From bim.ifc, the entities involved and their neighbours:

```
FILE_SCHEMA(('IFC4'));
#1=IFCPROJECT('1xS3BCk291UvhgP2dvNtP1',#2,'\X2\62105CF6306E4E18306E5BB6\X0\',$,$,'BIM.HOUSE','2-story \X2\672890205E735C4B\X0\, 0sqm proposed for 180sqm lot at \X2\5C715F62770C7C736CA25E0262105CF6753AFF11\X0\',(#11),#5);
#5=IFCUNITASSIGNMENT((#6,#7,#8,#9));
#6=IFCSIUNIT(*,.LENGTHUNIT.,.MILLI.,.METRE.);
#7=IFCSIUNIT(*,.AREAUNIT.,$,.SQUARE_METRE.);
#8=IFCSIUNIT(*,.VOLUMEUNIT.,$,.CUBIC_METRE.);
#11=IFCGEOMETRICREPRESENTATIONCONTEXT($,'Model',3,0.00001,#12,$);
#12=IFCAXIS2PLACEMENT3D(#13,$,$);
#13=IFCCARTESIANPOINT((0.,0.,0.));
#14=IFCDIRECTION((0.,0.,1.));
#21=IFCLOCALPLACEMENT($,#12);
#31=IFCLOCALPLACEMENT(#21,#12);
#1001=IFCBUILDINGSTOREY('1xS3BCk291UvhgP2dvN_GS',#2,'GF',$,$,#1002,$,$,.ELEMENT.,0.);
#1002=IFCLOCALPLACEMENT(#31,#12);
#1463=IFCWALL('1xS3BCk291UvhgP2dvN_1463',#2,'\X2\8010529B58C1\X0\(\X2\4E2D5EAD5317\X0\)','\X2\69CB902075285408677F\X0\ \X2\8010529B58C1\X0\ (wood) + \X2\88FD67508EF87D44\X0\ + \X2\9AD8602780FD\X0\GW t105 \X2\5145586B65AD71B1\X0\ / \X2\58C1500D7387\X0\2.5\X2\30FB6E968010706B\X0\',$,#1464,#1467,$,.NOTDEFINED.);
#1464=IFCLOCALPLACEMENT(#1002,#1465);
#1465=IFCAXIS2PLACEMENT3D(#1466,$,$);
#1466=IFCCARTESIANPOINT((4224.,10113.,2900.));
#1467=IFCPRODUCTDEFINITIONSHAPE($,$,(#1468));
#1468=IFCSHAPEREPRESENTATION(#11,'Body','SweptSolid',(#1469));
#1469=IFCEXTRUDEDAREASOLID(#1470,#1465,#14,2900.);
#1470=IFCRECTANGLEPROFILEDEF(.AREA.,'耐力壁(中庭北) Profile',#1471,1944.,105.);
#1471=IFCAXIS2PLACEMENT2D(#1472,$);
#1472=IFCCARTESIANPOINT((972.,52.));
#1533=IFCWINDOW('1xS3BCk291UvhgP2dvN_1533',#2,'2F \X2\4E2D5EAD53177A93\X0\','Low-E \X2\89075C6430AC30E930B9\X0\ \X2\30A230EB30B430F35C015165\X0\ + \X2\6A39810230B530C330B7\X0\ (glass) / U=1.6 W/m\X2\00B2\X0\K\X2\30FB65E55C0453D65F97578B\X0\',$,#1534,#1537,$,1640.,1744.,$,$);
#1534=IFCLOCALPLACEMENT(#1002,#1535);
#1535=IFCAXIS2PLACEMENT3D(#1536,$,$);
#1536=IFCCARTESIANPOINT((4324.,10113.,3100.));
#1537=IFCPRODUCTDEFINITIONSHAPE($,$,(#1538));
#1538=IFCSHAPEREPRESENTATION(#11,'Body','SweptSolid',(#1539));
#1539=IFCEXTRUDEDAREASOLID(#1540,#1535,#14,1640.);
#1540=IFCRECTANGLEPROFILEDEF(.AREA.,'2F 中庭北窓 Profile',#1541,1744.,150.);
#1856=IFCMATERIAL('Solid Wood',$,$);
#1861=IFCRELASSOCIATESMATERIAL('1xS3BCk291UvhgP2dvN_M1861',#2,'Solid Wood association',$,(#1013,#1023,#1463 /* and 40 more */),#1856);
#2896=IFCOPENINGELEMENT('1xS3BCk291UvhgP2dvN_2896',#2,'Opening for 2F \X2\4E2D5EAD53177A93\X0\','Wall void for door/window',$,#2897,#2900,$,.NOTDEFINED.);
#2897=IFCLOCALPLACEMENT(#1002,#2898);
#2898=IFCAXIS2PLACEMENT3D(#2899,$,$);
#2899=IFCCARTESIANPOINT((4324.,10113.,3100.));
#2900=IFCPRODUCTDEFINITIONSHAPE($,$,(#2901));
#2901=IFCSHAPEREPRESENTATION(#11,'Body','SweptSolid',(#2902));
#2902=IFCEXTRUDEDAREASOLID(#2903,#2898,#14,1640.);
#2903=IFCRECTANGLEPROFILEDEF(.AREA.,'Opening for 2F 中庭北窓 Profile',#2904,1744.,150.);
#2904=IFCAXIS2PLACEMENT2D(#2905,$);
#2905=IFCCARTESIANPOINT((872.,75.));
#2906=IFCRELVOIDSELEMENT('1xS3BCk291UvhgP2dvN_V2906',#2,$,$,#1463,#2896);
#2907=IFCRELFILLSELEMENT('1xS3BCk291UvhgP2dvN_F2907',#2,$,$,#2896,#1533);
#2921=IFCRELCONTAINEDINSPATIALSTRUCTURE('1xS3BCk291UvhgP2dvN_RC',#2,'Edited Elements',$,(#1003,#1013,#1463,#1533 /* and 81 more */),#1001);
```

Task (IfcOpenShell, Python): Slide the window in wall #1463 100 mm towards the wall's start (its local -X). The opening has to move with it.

```python
import ifcopenshell
import ifcopenshell.api.geometry
import ifcopenshell.util.placement

model = ifcopenshell.open("bim.ifc")

window = model.by_guid("1xS3BCk291UvhgP2dvN_1533")
opening = window.FillsVoids[0].RelatingOpeningElement
wall = opening.VoidsElements[0].RelatingBuildingElement

wall_matrix = ifcopenshell.util.placement.get_local_placement(wall.ObjectPlacement)
shift = wall_matrix[:3, 0] * -100.0
before = ifcopenshell.util.placement.get_local_placement(window.ObjectPlacement)[:3, 3].copy()

# The window is not placed relative to its opening, so move both.
for product in (opening, window):
    matrix = ifcopenshell.util.placement.get_local_placement(product.ObjectPlacement)
    matrix[:3, 3] += shift
    ifcopenshell.api.geometry.edit_object_placement(model, product=product, matrix=matrix, is_si=False)

after = ifcopenshell.util.placement.get_local_placement(window.ObjectPlacement)[:3, 3]
print("window moved by", (after - before).round(3) + 0.0)

model.write("bim_rev.ifc")
```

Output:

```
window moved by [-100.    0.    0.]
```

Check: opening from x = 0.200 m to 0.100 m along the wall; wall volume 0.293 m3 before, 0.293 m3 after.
